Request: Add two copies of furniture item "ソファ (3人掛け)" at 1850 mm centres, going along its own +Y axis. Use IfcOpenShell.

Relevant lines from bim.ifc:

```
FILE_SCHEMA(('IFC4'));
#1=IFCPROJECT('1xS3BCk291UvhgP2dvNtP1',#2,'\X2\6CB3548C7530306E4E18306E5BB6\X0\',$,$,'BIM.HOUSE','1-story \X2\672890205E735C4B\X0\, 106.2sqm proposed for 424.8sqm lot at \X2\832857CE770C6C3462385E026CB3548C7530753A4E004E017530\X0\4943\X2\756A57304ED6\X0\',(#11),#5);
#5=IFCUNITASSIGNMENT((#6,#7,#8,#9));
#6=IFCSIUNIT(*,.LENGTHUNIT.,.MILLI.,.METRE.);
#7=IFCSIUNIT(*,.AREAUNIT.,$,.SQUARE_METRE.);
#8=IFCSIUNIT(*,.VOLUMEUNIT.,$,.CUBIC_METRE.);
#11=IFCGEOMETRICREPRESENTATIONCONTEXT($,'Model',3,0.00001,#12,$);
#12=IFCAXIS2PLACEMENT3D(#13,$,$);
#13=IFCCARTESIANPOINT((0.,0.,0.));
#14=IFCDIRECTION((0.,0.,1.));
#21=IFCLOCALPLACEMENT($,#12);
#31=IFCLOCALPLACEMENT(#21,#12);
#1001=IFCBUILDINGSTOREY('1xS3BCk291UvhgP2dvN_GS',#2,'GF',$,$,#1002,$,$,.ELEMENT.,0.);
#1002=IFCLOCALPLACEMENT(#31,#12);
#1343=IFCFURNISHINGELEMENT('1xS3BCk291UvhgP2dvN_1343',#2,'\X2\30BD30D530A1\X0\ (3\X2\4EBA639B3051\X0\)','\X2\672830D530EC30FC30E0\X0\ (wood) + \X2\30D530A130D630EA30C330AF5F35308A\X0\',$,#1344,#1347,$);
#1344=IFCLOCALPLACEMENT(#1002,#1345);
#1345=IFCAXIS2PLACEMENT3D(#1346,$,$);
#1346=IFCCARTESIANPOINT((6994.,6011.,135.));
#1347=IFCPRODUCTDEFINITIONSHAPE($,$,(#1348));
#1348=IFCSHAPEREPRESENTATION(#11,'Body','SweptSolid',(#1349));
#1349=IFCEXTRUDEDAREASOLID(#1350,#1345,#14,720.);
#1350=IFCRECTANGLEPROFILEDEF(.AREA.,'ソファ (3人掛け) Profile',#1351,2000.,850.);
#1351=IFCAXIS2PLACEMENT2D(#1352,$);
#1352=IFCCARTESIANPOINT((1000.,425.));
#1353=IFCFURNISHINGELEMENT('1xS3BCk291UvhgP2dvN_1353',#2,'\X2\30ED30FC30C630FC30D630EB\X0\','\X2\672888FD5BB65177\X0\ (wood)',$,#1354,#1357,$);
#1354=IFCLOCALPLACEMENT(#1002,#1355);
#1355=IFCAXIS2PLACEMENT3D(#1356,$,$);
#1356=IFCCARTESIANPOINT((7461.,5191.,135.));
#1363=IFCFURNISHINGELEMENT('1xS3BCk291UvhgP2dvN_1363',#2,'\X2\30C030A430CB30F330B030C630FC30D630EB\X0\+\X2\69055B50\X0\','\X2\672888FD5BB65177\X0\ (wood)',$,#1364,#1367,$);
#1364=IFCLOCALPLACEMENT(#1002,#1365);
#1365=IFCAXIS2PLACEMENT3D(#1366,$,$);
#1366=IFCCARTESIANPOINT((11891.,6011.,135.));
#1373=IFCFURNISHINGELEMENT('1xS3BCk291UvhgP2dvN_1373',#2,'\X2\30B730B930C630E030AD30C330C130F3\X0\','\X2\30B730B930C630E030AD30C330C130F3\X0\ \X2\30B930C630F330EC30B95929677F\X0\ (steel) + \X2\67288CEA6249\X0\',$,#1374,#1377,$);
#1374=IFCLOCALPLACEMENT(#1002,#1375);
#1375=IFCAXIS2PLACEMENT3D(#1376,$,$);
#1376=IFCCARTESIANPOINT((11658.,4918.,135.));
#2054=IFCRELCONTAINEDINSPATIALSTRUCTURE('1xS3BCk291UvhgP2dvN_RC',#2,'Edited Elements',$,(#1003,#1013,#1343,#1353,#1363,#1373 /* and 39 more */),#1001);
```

```python
import ifcopenshell
import ifcopenshell.api.geometry
import ifcopenshell.api.root
import ifcopenshell.util.element
import ifcopenshell.util.placement

model = ifcopenshell.open("bim.ifc")


def reuse_history(source, copy):
    """copy_class also copies each property set's owner history, people and application; keep the originals."""
    for rel in copy.IsDefinedBy:
        if rel.is_a("IfcRelDefinesByProperties") and (history := rel.RelatingPropertyDefinition.OwnerHistory):
            rel.RelatingPropertyDefinition.OwnerHistory = source.OwnerHistory
            ifcopenshell.util.element.remove_deep2(model, history)


source = model.by_guid("1xS3BCk291UvhgP2dvN_1343")
base = ifcopenshell.util.placement.get_local_placement(source.ObjectPlacement)
step = base[:3, 1] * 1850.0

for i in range(1, 3):
    copy = ifcopenshell.api.root.copy_class(model, product=source)
    copy.Representation = ifcopenshell.util.element.copy_deep(
        model, source.Representation, exclude=["IfcGeometricRepresentationContext", "IfcRepresentationMap"]
    )
    reuse_history(source, copy)
    matrix = base.copy()
    matrix[:3, 3] += i * step
    print("added at", matrix[:3, 3].round(3) + 0.0)
    ifcopenshell.api.geometry.edit_object_placement(model, product=copy, matrix=matrix, is_si=False)

model.write("bim_edited.ifc")
```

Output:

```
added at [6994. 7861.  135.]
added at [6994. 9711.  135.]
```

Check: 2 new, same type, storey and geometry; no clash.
